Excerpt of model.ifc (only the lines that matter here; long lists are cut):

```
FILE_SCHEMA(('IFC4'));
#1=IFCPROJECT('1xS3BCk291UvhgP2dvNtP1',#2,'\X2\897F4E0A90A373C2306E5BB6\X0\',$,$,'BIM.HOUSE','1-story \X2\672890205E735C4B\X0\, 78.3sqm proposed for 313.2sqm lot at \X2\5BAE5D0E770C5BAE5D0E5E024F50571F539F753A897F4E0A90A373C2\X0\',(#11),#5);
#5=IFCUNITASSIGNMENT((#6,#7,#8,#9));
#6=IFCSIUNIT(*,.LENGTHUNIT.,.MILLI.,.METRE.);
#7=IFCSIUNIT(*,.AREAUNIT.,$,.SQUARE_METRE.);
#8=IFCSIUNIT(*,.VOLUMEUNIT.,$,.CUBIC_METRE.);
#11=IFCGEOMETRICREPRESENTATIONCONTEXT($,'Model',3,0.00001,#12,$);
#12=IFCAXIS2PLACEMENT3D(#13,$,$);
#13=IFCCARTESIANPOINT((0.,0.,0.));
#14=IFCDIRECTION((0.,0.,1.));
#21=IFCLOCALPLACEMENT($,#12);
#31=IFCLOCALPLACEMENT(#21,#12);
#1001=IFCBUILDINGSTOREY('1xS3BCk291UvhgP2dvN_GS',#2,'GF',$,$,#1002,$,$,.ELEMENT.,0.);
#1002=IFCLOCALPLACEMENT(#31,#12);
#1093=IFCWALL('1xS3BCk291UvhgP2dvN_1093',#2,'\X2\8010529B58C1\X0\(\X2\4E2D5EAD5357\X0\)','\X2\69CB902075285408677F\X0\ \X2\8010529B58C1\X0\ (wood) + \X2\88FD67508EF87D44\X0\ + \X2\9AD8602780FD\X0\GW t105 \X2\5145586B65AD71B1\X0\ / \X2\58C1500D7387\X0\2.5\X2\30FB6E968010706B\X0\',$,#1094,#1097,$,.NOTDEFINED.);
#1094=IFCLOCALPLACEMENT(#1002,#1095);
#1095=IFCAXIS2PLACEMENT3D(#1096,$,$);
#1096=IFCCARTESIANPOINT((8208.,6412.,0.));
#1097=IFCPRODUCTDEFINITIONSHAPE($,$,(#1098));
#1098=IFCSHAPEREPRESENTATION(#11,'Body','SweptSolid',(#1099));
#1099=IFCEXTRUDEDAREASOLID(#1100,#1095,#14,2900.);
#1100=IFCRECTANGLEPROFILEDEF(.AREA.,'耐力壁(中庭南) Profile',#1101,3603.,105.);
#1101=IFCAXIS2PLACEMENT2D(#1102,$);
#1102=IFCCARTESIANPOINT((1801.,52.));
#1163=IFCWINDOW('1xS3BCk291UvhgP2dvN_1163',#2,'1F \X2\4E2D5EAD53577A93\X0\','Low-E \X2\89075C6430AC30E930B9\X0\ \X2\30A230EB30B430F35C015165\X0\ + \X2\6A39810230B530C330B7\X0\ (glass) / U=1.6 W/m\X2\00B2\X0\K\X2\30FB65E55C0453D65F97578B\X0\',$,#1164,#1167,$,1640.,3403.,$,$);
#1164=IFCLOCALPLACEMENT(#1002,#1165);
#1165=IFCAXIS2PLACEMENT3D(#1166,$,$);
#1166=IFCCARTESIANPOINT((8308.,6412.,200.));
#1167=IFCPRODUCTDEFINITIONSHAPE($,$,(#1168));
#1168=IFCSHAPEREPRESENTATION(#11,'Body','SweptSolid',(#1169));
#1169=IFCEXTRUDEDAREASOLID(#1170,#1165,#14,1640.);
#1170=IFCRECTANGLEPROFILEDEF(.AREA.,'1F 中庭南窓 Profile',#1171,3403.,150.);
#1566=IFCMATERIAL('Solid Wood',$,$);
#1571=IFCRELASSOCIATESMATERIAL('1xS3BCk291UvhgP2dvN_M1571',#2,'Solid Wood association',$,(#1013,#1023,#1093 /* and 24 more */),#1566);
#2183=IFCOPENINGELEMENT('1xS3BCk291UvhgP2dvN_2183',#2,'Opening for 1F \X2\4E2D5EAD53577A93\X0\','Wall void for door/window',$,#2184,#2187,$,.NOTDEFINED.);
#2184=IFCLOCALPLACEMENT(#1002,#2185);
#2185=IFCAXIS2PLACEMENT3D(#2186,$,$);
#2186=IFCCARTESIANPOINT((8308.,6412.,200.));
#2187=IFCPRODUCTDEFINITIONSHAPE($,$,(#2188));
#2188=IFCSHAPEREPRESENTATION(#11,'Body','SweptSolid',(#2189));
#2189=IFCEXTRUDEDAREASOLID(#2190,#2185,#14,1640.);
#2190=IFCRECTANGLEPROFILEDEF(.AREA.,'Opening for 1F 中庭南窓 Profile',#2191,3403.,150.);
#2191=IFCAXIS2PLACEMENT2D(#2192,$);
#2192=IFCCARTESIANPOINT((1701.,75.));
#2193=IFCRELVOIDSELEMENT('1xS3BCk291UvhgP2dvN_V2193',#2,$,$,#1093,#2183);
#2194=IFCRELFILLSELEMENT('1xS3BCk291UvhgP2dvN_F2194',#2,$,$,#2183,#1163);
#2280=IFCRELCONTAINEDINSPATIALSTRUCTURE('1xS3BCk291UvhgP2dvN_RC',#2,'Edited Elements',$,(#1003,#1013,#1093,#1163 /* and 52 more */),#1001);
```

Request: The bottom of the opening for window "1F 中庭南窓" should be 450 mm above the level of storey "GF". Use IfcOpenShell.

```python
import numpy as np
import ifcopenshell
import ifcopenshell.api.geometry
import ifcopenshell.geom
import ifcopenshell.util.element
import ifcopenshell.util.placement
import ifcopenshell.util.shape
import ifcopenshell.util.unit

model = ifcopenshell.open("model.ifc")
unit_scale = ifcopenshell.util.unit.calculate_unit_scale(model)

window = model.by_id(1163)
opening = window.FillsVoids[0].RelatingOpeningElement
storey = ifcopenshell.util.element.get_container(window, ifc_class="IfcBuildingStorey")
level = ifcopenshell.util.placement.get_local_placement(storey.ObjectPlacement)[2, 3]

# The opening's origin need not be at the sill, so measure its lowest point.
shape = ifcopenshell.geom.create_shape(ifcopenshell.geom.settings(), opening)
bottom = ifcopenshell.util.shape.get_shape_bottom_elevation(shape, shape.geometry) / unit_scale
dz = level + 0.45 / unit_scale - bottom

shift = np.array([0.0, 0.0, dz])
# The window is not placed relative to its opening, so move both.
for product in (opening, window):
    matrix = ifcopenshell.util.placement.get_local_placement(product.ObjectPlacement)
    matrix[:3, 3] += shift
    ifcopenshell.api.geometry.edit_object_placement(model, product=product, matrix=matrix, is_si=False)

print(f"moved by {dz * unit_scale:+.3f} m")

model.write("model_v2.ifc")
```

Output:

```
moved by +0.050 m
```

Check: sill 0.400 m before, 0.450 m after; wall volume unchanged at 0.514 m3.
